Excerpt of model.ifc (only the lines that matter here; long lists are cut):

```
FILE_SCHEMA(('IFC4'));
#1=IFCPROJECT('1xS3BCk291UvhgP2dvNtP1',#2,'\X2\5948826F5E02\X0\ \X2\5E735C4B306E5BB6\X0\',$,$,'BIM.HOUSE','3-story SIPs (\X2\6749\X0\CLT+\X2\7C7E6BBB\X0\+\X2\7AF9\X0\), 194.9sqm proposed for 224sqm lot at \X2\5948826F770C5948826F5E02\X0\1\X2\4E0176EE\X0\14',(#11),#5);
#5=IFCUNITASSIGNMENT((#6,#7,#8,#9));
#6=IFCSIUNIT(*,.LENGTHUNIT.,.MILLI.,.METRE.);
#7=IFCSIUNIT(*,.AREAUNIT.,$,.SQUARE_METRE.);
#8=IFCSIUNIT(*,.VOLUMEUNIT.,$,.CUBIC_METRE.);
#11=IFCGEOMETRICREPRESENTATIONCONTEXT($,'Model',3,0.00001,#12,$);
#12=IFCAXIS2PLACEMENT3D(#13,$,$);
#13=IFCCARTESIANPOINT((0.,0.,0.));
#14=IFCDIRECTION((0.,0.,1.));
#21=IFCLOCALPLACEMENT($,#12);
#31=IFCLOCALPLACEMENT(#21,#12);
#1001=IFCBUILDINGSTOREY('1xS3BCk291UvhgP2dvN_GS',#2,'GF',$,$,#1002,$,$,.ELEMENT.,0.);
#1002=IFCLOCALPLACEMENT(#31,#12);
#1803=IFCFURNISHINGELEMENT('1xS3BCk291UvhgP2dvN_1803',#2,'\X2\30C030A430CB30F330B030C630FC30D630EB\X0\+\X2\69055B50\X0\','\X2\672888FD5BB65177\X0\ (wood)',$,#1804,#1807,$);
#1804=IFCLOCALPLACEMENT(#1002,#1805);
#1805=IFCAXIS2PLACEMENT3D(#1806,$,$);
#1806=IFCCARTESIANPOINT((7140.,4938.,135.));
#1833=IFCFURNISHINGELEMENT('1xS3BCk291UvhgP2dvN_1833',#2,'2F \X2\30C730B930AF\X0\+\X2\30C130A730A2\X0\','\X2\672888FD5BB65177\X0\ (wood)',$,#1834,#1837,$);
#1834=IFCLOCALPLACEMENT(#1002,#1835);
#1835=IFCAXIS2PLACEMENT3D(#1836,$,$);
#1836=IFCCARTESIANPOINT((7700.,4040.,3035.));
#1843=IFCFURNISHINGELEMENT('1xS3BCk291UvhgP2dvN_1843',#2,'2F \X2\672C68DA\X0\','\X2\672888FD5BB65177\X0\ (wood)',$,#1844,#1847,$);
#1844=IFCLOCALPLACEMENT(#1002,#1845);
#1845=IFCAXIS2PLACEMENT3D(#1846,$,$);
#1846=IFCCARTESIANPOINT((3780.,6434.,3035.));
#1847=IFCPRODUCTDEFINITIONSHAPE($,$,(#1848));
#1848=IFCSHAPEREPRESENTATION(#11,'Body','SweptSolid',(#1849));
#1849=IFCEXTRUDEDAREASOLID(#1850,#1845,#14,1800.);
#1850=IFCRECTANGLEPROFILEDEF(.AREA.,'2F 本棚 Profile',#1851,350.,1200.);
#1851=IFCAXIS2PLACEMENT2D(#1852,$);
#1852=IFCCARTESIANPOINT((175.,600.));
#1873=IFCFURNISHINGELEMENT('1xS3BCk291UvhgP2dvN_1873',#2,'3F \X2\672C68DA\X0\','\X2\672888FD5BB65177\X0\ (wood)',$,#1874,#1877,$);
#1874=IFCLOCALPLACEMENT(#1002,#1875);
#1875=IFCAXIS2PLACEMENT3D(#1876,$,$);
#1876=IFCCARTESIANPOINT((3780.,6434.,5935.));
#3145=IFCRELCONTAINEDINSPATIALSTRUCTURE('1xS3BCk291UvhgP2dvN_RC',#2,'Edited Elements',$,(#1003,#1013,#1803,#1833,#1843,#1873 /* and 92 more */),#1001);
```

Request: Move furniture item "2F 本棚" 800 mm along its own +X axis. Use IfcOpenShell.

```python
import ifcopenshell
import ifcopenshell.api.geometry
import ifcopenshell.util.placement

model = ifcopenshell.open("model.ifc")

item = model.by_id(1843)
matrix = ifcopenshell.util.placement.get_local_placement(item.ObjectPlacement)
matrix[:3, 3] += matrix[:3, 0] * 800.0
ifcopenshell.api.geometry.edit_object_placement(model, product=item, matrix=matrix, is_si=False)

print(ifcopenshell.util.placement.get_local_placement(item.ObjectPlacement).round(3) + 0.0)

model.write("model_edited.ifc")
```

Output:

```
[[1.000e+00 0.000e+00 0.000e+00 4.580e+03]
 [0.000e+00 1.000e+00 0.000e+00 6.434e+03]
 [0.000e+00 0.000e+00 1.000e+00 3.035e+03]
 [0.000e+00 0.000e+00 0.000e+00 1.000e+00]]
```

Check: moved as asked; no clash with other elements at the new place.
